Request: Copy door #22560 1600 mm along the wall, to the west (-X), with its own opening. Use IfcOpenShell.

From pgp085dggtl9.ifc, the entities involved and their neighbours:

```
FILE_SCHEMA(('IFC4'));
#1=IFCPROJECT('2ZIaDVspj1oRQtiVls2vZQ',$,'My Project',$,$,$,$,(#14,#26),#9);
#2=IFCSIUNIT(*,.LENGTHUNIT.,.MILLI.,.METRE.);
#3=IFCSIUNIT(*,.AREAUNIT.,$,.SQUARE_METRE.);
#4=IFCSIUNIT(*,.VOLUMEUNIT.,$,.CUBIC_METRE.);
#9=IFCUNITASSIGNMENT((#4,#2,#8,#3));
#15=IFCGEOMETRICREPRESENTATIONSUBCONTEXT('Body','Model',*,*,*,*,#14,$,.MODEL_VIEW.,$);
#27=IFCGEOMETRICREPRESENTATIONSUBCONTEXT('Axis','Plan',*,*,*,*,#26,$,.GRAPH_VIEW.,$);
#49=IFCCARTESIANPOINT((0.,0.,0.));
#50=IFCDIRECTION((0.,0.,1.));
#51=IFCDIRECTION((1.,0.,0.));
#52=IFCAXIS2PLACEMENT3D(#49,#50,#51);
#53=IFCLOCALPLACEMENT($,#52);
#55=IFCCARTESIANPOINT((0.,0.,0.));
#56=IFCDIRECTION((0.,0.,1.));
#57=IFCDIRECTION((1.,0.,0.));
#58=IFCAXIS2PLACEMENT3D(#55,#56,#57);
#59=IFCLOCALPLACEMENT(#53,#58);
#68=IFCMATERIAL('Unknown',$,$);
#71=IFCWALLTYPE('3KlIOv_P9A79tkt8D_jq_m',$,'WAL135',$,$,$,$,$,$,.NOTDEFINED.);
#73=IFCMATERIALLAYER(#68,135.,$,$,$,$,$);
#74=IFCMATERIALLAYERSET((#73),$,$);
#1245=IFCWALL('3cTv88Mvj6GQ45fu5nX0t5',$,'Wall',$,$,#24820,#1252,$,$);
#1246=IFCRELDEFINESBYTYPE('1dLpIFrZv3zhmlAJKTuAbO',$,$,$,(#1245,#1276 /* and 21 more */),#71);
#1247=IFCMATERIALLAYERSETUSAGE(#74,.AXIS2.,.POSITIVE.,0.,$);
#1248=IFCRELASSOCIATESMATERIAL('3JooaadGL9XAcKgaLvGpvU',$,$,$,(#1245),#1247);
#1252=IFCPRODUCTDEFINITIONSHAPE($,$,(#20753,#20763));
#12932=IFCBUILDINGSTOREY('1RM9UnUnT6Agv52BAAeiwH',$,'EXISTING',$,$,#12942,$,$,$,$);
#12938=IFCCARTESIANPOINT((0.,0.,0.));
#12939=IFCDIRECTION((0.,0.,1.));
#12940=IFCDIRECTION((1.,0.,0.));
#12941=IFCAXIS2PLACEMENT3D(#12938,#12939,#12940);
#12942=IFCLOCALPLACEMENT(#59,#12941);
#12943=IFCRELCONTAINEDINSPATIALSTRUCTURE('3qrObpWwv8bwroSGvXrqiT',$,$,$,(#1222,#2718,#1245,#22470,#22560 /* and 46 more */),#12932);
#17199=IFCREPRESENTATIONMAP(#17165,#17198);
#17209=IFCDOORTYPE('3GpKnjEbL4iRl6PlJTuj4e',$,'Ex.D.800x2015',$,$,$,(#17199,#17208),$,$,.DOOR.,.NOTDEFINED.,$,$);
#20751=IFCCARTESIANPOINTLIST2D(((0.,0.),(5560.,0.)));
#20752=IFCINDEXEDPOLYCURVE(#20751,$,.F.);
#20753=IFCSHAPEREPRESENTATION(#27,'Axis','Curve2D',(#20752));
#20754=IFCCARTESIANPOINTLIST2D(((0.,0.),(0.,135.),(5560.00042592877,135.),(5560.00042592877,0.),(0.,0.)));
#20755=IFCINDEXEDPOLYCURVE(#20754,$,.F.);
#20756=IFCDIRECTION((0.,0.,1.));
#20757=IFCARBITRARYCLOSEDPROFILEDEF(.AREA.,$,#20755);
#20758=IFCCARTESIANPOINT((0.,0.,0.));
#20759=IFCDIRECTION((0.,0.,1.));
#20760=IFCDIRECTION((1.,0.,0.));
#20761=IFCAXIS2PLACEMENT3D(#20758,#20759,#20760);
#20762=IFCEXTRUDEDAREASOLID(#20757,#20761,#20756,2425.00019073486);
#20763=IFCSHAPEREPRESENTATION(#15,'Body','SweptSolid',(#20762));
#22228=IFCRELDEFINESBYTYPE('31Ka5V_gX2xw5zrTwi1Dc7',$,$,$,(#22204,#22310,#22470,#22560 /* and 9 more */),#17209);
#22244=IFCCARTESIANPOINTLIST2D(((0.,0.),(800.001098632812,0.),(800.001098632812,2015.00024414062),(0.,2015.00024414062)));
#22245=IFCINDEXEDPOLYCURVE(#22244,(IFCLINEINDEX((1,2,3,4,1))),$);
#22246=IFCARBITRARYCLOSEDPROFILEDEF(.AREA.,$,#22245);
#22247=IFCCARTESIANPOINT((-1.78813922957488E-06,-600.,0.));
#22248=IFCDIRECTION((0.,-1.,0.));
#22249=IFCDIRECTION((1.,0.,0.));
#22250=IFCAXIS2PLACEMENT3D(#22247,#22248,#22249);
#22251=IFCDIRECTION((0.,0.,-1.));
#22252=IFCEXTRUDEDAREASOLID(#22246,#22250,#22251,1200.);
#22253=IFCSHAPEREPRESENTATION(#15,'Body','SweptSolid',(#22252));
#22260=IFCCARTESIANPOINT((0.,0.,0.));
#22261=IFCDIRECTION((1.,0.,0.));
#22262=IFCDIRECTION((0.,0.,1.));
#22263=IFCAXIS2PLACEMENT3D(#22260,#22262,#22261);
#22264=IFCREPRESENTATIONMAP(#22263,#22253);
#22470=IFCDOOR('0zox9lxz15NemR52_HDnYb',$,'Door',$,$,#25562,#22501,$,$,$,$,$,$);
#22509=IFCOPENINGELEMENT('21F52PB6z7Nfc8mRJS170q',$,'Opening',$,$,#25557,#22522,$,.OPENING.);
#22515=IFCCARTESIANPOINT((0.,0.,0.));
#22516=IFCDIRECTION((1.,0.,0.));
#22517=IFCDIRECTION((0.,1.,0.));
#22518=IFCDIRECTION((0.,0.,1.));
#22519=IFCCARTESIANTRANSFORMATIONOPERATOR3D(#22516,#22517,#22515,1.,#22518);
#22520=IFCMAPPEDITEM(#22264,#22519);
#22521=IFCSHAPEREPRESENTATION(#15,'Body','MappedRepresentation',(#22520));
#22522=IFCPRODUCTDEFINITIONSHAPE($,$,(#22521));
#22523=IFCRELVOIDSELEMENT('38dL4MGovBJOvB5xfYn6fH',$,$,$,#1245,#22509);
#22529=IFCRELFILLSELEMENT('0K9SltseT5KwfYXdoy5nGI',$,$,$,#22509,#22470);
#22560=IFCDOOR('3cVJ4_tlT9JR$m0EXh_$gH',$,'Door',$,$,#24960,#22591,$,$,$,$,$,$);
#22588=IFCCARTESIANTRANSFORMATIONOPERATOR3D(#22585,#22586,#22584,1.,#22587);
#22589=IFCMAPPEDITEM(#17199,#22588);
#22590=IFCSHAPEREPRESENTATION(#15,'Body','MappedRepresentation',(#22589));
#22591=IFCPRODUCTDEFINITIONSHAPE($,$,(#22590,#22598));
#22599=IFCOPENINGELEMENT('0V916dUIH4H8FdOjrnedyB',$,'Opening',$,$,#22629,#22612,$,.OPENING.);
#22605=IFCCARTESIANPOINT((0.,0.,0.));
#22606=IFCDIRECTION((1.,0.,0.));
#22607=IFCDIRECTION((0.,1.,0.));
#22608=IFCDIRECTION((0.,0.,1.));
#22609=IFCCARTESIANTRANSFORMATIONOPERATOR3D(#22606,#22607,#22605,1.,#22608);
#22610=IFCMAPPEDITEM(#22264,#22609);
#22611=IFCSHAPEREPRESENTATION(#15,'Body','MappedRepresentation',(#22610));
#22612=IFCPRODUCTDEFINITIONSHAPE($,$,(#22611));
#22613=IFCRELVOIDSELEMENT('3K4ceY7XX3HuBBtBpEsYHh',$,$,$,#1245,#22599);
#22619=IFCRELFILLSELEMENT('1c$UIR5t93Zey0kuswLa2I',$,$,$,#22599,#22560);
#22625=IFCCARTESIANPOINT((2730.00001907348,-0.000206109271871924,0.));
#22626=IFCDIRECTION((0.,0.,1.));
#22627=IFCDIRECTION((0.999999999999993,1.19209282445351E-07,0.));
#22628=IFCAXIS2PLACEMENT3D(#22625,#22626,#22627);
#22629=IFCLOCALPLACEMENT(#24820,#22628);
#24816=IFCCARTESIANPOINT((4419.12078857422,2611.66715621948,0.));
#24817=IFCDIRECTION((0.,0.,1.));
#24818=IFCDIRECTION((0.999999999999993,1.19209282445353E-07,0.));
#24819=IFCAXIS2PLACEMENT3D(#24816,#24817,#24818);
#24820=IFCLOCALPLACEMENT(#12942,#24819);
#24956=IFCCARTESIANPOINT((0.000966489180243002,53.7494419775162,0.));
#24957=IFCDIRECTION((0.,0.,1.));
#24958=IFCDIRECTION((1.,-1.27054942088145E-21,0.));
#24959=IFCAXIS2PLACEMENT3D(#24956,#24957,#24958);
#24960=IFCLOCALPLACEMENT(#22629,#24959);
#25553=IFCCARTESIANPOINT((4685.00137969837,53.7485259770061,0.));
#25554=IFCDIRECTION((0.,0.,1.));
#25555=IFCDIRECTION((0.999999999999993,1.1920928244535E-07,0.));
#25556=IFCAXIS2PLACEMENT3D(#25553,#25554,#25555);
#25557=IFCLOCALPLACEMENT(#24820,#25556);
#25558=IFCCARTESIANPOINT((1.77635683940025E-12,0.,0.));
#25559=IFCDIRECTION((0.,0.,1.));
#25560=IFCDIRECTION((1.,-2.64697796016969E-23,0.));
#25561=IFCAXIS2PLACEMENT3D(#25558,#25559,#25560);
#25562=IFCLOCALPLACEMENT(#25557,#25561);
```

```python
import ifcopenshell
import ifcopenshell.api.feature
import ifcopenshell.api.geometry
import ifcopenshell.api.root
import ifcopenshell.geom
import ifcopenshell.util.element
import ifcopenshell.util.placement
import ifcopenshell.util.shape

model = ifcopenshell.open("pgp085dggtl9.ifc")
settings = ifcopenshell.geom.settings()


def volume(element):
    """Net volume in cubic metres, openings subtracted."""
    shape = ifcopenshell.geom.create_shape(settings, element)
    return ifcopenshell.util.shape.get_volume(shape.geometry)


door = model.by_guid("3cVJ4_tlT9JR$m0EXh_$gH")
opening = door.FillsVoids[0].RelatingOpeningElement
wall = opening.VoidsElements[0].RelatingBuildingElement
before = volume(wall)
shift = ifcopenshell.util.placement.get_local_placement(wall.ObjectPlacement)[:3, 0] * -1600.0

# copy_class copies the void relationship, type, container and properties, but no geometry.
new_opening = ifcopenshell.api.root.copy_class(model, product=opening)
new_opening.Representation = ifcopenshell.util.element.copy_deep(
    model, opening.Representation, exclude=["IfcGeometricRepresentationContext", "IfcRepresentationMap"]
)
new_door = ifcopenshell.api.root.copy_class(model, product=door)
new_door.Representation = ifcopenshell.util.element.copy_deep(
    model, door.Representation, exclude=["IfcGeometricRepresentationContext", "IfcRepresentationMap"]
)
ifcopenshell.api.feature.add_filling(model, opening=new_opening, element=new_door)

for old, new in ((opening, new_opening), (door, new_door)):
    matrix = ifcopenshell.util.placement.get_local_placement(old.ObjectPlacement)
    matrix[:3, 3] += shift
    ifcopenshell.api.geometry.edit_object_placement(model, product=new, matrix=matrix, is_si=False)

after = volume(wall)

print(f"wall volume {before:.3f} -> {after:.3f} m3")

model.write("pgp085dggtl9_updated.ifc")
```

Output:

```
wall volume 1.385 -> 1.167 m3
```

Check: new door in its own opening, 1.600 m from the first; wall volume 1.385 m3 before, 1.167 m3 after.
